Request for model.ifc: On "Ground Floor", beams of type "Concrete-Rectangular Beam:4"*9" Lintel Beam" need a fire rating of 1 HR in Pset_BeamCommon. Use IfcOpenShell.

First a look at what the model holds.

```python
import ifcopenshell
import ifcopenshell.util.element

model = ifcopenshell.open("model.ifc")
print(model.schema)
storey = next(s for s in model.by_type("IfcBuildingStorey") if s.Name == "Ground Floor")
beams = [e for e in ifcopenshell.util.element.get_decomposition(storey) if e.is_a("IfcBeam")]
seen = {}
for e in beams:
    element_type = ifcopenshell.util.element.get_type(e)
    key = (element_type.Name if element_type != e and element_type else None, ifcopenshell.util.element.get_pset(e, "Pset_BeamCommon", "FireRating"))
    seen[key] = seen.get(key, 0) + 1
for (name, value), count in sorted(seen.items(), key=str):
    print(count, "x", name, "|", value)
```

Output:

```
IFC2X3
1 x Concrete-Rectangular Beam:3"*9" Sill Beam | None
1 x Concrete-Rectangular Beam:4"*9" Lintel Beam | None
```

```python
import ifcopenshell
import ifcopenshell.api.pset
import ifcopenshell.util.element

model = ifcopenshell.open("model.ifc")

storey = next(s for s in model.by_type("IfcBuildingStorey") if s.Name == "Ground Floor")
beams = [e for e in ifcopenshell.util.element.get_decomposition(storey) if e.is_a("IfcBeam")]

count = 0
for e in beams:
    element_type = ifcopenshell.util.element.get_type(e)
    if element_type in (None, e) or element_type.Name != 'Concrete-Rectangular Beam:4"*9" Lintel Beam':
        continue
    # add_pset returns the element's existing set when there is one.
    pset = ifcopenshell.api.pset.add_pset(model, product=e, name="Pset_BeamCommon")
    ifcopenshell.api.pset.edit_pset(model, pset=pset, properties={"FireRating": "1 HR"})
    count += 1

print(count, "beams updated")

model.write("model_edited.ifc")
```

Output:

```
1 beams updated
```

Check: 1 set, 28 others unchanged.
